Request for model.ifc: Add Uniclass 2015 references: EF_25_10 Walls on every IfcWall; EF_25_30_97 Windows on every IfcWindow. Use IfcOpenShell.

First a look at what the model holds.

```python
import ifcopenshell

model = ifcopenshell.open("model.ifc")
print(model.schema)
print("classifications:", [c.Name for c in model.by_type("IfcClassification")])
for ifc_class in ("IfcDoor", "IfcRoof", "IfcStair", "IfcWall", "IfcWindow"):
    print(ifc_class, len(model.by_type(ifc_class)))
```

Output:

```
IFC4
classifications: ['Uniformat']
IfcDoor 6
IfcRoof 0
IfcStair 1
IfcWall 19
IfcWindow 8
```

```python
import ifcopenshell
import ifcopenshell.api.classification

model = ifcopenshell.open("model.ifc")

system = ifcopenshell.api.classification.add_classification(model, classification="Uniclass 2015")

codes = {
    "IfcWall": ("EF_25_10", "Walls"),
    "IfcWindow": ("EF_25_30_97", "Windows"),
}
for ifc_class, (code, name) in codes.items():
    products = model.by_type(ifc_class)
    ifcopenshell.api.classification.add_reference(
        model, products=products, classification=system, identification=code, name=name
    )
    print(code, len(products))

model.write("model-out.ifc")
```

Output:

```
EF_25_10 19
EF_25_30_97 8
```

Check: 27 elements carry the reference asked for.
